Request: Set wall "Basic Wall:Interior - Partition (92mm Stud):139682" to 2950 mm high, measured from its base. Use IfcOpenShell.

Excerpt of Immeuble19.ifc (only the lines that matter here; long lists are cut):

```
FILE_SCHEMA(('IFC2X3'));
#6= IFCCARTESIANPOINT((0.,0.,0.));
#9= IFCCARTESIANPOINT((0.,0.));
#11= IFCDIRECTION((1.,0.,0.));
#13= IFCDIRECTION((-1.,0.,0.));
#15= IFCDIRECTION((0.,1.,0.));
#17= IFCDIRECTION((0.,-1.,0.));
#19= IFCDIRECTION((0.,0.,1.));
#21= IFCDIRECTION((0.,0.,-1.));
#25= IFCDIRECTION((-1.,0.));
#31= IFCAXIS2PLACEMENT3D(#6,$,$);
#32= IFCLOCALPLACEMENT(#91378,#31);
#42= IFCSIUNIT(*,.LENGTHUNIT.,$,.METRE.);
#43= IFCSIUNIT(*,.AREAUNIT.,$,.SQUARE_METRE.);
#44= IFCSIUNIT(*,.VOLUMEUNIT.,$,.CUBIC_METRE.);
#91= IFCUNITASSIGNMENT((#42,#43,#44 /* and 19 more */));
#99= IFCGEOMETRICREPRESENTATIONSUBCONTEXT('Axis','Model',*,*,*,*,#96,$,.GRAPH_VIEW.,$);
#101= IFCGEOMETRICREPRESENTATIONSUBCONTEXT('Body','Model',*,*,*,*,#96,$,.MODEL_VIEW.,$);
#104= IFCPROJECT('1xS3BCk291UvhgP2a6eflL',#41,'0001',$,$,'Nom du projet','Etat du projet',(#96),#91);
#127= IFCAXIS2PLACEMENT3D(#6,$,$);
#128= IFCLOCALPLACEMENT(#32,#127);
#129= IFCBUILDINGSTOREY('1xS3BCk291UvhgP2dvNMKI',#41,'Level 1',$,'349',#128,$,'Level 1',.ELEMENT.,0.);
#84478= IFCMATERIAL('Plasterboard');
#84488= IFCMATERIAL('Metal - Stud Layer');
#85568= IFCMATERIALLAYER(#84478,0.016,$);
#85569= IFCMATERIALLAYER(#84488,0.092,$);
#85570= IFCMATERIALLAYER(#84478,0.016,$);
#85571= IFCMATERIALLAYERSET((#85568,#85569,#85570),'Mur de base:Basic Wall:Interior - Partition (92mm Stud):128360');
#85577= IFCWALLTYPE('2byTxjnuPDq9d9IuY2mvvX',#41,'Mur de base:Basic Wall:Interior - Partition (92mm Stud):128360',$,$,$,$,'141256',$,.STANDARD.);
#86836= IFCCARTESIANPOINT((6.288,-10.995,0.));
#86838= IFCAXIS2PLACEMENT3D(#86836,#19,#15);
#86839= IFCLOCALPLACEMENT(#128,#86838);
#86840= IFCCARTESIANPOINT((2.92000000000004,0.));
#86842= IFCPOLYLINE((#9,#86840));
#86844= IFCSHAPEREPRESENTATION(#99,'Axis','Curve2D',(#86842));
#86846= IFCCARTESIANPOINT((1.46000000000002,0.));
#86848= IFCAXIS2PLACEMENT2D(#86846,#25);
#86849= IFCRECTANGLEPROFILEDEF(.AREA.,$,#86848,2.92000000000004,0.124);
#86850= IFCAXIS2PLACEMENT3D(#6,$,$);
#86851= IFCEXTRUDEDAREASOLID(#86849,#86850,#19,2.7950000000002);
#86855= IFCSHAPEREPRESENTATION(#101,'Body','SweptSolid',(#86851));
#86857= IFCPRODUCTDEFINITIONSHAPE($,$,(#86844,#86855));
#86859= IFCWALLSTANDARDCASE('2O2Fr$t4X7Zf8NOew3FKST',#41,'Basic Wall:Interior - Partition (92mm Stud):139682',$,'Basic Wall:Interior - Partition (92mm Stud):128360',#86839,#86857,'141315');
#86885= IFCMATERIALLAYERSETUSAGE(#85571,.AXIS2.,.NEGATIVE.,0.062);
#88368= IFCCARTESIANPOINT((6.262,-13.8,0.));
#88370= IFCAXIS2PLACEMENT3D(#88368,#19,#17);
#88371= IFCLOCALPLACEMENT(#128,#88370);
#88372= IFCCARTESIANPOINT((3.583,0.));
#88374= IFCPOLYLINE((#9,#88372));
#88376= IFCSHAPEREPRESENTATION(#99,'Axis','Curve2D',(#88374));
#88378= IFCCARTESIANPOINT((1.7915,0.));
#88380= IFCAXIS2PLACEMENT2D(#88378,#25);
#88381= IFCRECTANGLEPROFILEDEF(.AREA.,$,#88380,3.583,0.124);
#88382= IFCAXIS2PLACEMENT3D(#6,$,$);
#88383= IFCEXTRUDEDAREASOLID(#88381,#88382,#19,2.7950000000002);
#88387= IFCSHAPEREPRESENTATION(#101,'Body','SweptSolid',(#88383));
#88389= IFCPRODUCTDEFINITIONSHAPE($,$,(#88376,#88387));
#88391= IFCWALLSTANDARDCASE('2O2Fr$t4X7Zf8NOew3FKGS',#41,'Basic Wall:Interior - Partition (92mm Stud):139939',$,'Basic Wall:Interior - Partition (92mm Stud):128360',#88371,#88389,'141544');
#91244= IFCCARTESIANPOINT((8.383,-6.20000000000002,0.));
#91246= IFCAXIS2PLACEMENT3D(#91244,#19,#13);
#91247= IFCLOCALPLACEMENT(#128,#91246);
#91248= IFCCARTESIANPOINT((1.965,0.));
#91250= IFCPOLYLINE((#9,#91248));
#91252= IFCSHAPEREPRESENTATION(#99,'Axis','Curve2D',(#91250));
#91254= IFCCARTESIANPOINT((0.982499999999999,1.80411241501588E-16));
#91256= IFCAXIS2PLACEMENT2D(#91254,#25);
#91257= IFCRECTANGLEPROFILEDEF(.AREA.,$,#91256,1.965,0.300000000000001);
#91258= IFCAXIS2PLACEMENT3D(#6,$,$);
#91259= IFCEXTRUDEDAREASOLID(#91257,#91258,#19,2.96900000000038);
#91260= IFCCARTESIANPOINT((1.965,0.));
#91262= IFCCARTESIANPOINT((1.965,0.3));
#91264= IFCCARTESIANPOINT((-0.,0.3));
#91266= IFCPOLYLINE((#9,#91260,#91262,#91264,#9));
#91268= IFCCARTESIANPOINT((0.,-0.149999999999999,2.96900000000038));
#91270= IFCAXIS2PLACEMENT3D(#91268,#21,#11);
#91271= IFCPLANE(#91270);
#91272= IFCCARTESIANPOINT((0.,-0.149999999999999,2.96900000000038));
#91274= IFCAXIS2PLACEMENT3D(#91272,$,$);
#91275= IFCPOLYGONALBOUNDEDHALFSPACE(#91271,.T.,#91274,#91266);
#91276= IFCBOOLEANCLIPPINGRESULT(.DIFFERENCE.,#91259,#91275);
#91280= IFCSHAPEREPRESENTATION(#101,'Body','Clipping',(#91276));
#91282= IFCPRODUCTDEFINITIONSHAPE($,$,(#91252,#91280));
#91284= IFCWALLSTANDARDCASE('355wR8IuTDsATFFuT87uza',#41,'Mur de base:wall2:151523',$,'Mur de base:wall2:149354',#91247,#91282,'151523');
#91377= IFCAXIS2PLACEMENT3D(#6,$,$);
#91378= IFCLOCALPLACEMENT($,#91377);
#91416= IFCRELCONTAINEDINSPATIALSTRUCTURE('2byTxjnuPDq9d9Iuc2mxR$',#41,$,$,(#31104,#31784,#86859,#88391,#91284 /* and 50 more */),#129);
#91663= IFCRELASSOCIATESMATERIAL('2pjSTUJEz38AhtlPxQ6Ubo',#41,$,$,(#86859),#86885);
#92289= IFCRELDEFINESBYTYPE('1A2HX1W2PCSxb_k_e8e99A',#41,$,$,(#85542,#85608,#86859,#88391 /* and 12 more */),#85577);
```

```python
import ifcopenshell
import ifcopenshell.geom
import ifcopenshell.util.representation
import ifcopenshell.util.shape

model = ifcopenshell.open("Immeuble19.ifc")
settings = ifcopenshell.geom.settings()


def volume(element):
    """Net volume in cubic metres, openings subtracted."""
    shape = ifcopenshell.geom.create_shape(settings, element)
    return ifcopenshell.util.shape.get_volume(shape.geometry)


wall = model.by_id(86859)
before = volume(wall)

body = ifcopenshell.util.representation.get_representation(wall, "Model", "Body")
solid = body.Items[0]
old_height = solid.Depth
solid.Depth = 2.95
after = volume(wall)

print(f"height {old_height:g} -> {solid.Depth:g}, volume {before:.3f} -> {after:.3f} m3")

model.write("Immeuble19_edited.ifc")
```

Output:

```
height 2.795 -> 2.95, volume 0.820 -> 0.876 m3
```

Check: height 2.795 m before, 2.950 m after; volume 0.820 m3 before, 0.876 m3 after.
